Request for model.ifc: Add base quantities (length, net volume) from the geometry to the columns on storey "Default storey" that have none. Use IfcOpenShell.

First a look at what the model holds.

```python
import ifcopenshell
import ifcopenshell.util.element
import ifcopenshell.util.unit

model = ifcopenshell.open("model.ifc")
print(model.schema)
for unit_type in ("LENGTHUNIT", "AREAUNIT", "VOLUMEUNIT"):
    print(unit_type, ifcopenshell.util.unit.calculate_unit_scale(model, unit_type))
storey = next(s for s in model.by_type("IfcBuildingStorey") if s.Name == "Default storey")
columns = [e for e in ifcopenshell.util.element.get_decomposition(storey) if e.is_a("IfcColumn")]
for e in sorted(columns, key=lambda e: e.id()):
    print(e.id(), e.is_a(), e.Name, list(ifcopenshell.util.element.get_psets(e, qtos_only=True)), sep=" | ")
```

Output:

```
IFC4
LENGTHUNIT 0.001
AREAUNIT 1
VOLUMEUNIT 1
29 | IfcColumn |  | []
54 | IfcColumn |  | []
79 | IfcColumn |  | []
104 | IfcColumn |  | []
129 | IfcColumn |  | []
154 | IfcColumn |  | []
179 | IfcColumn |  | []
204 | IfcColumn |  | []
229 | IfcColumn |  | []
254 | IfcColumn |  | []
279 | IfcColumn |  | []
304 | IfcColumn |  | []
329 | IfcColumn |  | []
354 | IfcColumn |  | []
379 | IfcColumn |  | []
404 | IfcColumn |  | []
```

```python
import ifcopenshell
import ifcopenshell.api.pset
import ifcopenshell.geom
import ifcopenshell.util.element
import ifcopenshell.util.shape
import ifcopenshell.util.unit

model = ifcopenshell.open("model.ifc")
unit_scale = ifcopenshell.util.unit.calculate_unit_scale(model)
volume_scale = ifcopenshell.util.unit.calculate_unit_scale(model, "VOLUMEUNIT")
settings = ifcopenshell.geom.settings()

storey = next(s for s in model.by_type("IfcBuildingStorey") if s.Name == "Default storey")
columns = [e for e in ifcopenshell.util.element.get_decomposition(storey) if e.is_a("IfcColumn")]

for e in sorted(columns, key=lambda e: e.id()):
    if ifcopenshell.util.element.get_psets(e, qtos_only=True, should_inherit=False):
        continue
    # Geometry comes back in metres, in the element's own axes.
    shape = ifcopenshell.geom.create_shape(settings, e)
    values = {
        "Length": ifcopenshell.util.shape.get_z(shape.geometry) / unit_scale,
        "NetVolume": ifcopenshell.util.shape.get_volume(shape.geometry) / volume_scale,
    }
    qto = ifcopenshell.api.pset.add_qto(model, product=e, name="Qto_ColumnBaseQuantities")
    ifcopenshell.api.pset.edit_qto(model, qto=qto, properties=values)
    print(e.id(), {k: round(v, 3) for k, v in values.items()})

model.write("model_v2.ifc")
```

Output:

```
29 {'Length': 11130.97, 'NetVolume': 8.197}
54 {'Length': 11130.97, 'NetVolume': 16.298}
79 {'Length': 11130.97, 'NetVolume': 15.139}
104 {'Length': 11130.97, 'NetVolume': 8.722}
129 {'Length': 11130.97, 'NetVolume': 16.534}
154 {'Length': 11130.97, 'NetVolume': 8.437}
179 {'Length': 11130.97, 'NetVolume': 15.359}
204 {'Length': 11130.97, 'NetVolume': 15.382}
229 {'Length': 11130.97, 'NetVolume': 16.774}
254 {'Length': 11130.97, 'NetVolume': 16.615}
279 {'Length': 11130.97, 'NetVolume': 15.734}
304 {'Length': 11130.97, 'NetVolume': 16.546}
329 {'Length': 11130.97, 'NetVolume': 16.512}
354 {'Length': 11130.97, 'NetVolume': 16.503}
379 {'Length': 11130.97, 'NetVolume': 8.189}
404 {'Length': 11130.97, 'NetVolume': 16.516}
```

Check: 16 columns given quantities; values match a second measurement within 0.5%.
